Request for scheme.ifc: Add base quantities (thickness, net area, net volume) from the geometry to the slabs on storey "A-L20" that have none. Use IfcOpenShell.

First a look at what the model holds.

```python
import ifcopenshell
import ifcopenshell.util.element
import ifcopenshell.util.unit

model = ifcopenshell.open("scheme.ifc")
print(model.schema)
for unit_type in ("LENGTHUNIT", "AREAUNIT", "VOLUMEUNIT"):
    print(unit_type, ifcopenshell.util.unit.calculate_unit_scale(model, unit_type))
storey = next(s for s in model.by_type("IfcBuildingStorey") if s.Name == "A-L20")
slabs = [e for e in ifcopenshell.util.element.get_decomposition(storey) if e.is_a("IfcSlab")]
for e in sorted(slabs, key=lambda e: e.id()):
    print(e.id(), e.is_a(), e.Name, list(ifcopenshell.util.element.get_psets(e, qtos_only=True)), sep=" | ")
```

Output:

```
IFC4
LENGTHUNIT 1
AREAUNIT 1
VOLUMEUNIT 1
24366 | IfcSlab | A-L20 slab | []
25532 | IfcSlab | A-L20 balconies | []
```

```python
import ifcopenshell
import ifcopenshell.api.pset
import ifcopenshell.geom
import ifcopenshell.util.element
import ifcopenshell.util.shape
import ifcopenshell.util.unit

model = ifcopenshell.open("scheme.ifc")
unit_scale = ifcopenshell.util.unit.calculate_unit_scale(model)
area_scale = ifcopenshell.util.unit.calculate_unit_scale(model, "AREAUNIT")
volume_scale = ifcopenshell.util.unit.calculate_unit_scale(model, "VOLUMEUNIT")
settings = ifcopenshell.geom.settings()

storey = next(s for s in model.by_type("IfcBuildingStorey") if s.Name == "A-L20")
slabs = [e for e in ifcopenshell.util.element.get_decomposition(storey) if e.is_a("IfcSlab")]

for e in sorted(slabs, key=lambda e: e.id()):
    if ifcopenshell.util.element.get_psets(e, qtos_only=True, should_inherit=False):
        continue
    # Geometry comes back in metres, in the element's own axes.
    shape = ifcopenshell.geom.create_shape(settings, e)
    values = {
        "Width": ifcopenshell.util.shape.get_z(shape.geometry) / unit_scale,
        "NetArea": ifcopenshell.util.shape.get_footprint_area(shape.geometry) / area_scale,
        "NetVolume": ifcopenshell.util.shape.get_volume(shape.geometry) / volume_scale,
    }
    qto = ifcopenshell.api.pset.add_qto(model, product=e, name="Qto_SlabBaseQuantities")
    ifcopenshell.api.pset.edit_qto(model, qto=qto, properties=values)
    print(e.id(), {k: round(v, 3) for k, v in values.items()})

model.write("scheme-out.ifc")
```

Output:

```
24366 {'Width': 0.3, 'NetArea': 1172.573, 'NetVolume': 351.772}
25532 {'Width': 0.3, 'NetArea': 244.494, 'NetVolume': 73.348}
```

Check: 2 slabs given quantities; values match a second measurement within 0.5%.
